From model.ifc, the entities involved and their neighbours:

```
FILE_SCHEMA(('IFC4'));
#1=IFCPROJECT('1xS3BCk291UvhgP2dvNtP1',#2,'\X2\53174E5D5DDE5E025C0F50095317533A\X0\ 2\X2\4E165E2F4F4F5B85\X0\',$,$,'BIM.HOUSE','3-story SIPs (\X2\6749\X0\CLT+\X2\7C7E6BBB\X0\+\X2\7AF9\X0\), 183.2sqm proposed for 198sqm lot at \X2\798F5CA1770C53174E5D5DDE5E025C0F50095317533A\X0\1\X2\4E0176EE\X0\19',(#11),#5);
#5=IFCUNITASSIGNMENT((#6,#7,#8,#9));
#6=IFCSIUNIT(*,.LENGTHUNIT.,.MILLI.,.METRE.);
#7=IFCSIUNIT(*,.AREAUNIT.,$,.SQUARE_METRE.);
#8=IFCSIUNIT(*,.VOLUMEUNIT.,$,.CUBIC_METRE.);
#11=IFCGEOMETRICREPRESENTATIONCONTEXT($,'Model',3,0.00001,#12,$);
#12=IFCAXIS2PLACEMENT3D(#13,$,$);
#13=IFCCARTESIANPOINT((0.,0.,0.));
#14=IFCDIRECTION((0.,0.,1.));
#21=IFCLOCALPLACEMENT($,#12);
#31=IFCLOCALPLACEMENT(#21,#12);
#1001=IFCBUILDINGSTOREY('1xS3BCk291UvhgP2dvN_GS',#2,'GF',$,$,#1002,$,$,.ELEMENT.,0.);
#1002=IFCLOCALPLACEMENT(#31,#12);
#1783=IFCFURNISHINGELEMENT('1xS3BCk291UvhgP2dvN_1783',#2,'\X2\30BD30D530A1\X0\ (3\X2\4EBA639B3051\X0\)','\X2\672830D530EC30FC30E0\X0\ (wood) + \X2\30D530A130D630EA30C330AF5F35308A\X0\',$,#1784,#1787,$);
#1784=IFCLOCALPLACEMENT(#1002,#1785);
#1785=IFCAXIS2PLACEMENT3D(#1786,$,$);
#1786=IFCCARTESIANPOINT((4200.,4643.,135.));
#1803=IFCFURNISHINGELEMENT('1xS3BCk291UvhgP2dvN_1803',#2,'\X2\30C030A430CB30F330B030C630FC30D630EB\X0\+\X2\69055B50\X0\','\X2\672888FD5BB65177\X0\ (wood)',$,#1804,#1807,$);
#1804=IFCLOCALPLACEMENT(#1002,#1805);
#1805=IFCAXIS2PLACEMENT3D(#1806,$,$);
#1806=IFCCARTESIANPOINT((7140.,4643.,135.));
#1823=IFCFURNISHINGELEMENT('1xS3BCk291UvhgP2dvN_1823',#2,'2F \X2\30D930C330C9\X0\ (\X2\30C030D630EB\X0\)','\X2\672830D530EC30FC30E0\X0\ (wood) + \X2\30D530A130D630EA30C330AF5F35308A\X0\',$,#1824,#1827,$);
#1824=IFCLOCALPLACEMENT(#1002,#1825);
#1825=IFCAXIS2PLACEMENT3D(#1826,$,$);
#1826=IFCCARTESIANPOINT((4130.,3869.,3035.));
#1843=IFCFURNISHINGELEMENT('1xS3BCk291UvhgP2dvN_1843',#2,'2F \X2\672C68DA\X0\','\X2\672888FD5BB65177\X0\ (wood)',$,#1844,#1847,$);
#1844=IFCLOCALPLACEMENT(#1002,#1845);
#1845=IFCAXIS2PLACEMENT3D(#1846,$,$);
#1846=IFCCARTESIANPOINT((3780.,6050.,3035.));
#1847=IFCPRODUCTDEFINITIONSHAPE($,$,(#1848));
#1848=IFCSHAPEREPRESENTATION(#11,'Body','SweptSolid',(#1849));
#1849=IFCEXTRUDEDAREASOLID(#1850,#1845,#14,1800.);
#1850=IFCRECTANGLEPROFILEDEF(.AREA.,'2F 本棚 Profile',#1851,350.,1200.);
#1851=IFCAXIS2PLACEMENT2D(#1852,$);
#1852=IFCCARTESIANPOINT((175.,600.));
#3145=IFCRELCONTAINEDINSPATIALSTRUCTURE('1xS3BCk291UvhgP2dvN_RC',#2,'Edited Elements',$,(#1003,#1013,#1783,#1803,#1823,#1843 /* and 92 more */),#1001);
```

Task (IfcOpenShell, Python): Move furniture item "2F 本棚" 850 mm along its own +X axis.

```python
import ifcopenshell
import ifcopenshell.api.geometry
import ifcopenshell.util.placement
import ifcopenshell.util.unit

model = ifcopenshell.open("model.ifc")
unit_scale = ifcopenshell.util.unit.calculate_unit_scale(model)

item = model.by_guid("1xS3BCk291UvhgP2dvN_1843")
matrix = ifcopenshell.util.placement.get_local_placement(item.ObjectPlacement)
matrix[:3, 3] += matrix[:3, 0] * 0.85 / unit_scale
ifcopenshell.api.geometry.edit_object_placement(model, product=item, matrix=matrix, is_si=False)

print(ifcopenshell.util.placement.get_local_placement(item.ObjectPlacement).round(3) + 0.0)

model.write("model_rev.ifc")
```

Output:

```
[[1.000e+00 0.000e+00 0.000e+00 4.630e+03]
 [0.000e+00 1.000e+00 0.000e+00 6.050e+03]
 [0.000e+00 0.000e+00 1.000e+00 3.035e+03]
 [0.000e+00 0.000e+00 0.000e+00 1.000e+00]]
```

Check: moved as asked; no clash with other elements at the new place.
